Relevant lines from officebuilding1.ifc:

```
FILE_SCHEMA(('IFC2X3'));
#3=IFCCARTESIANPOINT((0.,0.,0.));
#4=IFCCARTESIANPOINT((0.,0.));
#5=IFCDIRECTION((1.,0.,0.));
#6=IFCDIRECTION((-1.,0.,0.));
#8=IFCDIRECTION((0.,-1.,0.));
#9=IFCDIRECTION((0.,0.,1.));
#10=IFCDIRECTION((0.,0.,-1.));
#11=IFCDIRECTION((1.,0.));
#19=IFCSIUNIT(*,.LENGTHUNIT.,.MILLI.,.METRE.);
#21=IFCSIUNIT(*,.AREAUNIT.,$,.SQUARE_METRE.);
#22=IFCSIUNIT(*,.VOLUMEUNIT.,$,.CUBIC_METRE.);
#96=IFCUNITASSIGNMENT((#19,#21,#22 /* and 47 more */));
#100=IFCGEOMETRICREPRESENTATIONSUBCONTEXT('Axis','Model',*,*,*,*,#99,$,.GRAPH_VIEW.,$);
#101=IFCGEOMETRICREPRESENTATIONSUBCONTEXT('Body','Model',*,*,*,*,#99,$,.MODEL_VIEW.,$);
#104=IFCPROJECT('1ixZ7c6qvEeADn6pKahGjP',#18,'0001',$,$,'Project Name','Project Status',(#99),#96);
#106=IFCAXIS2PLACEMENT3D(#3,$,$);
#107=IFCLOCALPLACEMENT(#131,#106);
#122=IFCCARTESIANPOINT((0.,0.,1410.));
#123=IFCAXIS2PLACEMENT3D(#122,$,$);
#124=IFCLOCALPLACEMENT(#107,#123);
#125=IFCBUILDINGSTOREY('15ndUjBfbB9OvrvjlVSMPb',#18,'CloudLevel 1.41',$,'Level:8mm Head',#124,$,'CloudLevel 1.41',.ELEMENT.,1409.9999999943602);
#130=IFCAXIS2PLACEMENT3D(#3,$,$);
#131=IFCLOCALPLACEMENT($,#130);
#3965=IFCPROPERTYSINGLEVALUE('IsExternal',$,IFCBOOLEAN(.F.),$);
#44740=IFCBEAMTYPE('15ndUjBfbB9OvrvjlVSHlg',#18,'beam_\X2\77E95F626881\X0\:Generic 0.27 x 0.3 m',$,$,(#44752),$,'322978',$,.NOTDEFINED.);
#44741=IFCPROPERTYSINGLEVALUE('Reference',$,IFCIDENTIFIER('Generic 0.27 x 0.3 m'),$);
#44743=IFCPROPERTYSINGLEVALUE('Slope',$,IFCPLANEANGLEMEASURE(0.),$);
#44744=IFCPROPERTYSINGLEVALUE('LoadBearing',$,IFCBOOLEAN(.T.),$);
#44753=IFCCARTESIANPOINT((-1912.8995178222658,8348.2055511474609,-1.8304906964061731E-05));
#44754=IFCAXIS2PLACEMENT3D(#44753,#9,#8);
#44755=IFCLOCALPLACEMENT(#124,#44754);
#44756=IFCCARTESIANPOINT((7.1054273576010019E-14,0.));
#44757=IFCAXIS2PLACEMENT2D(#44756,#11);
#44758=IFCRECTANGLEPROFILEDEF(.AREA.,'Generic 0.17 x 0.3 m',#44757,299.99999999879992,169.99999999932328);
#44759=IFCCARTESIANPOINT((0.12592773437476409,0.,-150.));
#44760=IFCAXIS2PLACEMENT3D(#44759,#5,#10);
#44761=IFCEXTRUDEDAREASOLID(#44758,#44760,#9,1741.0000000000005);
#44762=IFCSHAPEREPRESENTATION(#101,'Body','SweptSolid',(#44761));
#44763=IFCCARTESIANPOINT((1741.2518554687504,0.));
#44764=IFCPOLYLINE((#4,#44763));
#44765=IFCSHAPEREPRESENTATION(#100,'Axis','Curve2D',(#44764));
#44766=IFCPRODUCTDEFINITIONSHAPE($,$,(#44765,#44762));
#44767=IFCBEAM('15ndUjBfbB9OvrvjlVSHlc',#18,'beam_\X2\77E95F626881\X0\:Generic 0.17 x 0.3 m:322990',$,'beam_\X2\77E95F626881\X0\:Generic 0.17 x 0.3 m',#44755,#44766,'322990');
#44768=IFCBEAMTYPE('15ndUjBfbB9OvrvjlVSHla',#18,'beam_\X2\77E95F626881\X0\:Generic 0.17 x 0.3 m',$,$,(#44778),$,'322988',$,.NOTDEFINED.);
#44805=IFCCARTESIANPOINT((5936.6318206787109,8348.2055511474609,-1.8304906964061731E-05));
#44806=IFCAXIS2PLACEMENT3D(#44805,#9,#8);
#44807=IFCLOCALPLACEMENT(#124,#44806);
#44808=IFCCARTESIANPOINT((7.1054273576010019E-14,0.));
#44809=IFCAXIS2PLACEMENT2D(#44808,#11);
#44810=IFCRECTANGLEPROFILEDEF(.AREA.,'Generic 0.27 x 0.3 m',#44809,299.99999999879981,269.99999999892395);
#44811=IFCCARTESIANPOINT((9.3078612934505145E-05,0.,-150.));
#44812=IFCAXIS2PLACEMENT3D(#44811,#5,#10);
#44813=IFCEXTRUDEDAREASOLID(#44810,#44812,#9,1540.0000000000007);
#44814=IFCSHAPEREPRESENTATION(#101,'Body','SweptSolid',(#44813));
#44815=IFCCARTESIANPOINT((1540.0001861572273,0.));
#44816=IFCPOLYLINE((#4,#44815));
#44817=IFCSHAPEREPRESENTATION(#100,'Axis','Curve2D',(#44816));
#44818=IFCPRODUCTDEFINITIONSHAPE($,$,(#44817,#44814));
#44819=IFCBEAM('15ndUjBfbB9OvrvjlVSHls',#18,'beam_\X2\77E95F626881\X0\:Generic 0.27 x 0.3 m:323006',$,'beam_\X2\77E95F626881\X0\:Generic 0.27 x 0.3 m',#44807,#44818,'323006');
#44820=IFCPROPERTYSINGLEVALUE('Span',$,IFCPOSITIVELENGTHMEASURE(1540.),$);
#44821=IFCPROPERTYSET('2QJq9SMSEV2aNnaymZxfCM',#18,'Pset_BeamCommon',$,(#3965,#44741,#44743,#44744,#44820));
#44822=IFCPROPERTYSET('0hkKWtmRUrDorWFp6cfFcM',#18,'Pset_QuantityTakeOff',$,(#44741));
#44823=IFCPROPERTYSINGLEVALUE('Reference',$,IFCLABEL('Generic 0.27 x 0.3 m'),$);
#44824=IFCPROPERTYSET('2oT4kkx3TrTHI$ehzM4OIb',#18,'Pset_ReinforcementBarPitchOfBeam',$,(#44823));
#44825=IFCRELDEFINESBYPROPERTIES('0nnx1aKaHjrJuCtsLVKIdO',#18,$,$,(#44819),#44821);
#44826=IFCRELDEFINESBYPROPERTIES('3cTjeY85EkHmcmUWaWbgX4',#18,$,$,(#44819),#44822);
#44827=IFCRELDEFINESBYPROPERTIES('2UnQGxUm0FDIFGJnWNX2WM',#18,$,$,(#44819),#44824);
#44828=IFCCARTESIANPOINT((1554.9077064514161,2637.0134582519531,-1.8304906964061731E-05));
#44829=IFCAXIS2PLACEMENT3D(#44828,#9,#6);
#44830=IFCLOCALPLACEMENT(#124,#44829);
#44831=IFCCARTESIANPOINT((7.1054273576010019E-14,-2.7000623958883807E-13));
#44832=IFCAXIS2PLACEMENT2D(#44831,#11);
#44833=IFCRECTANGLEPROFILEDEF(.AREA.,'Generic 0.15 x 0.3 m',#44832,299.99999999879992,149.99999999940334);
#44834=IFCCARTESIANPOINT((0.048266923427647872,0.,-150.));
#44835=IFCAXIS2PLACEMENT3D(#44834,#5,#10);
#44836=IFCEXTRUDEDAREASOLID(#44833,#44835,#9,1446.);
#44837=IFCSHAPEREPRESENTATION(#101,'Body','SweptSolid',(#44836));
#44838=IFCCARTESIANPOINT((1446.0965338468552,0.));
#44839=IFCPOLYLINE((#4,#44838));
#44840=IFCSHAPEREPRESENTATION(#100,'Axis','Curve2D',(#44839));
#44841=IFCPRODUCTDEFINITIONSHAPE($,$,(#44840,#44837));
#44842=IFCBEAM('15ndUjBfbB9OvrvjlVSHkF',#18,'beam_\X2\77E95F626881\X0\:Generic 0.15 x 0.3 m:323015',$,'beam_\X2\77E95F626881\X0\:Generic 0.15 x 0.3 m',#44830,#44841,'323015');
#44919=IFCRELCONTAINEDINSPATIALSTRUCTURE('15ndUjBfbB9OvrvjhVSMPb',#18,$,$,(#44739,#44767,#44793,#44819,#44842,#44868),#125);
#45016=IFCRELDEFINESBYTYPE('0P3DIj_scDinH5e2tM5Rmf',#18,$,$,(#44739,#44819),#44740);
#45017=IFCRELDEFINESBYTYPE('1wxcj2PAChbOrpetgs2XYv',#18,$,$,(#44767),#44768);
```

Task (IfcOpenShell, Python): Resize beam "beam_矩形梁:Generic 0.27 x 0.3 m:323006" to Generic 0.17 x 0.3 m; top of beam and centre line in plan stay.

```python
import ifcopenshell
import ifcopenshell.api.pset
import ifcopenshell.api.type
import ifcopenshell.util.element
import ifcopenshell.util.representation

model = ifcopenshell.open("officebuilding1.ifc")

member = model.by_id(44819)
source = next(p for p in model.by_type("IfcRectangleProfileDef") if p.ProfileName == "Generic 0.17 x 0.3 m")

body = ifcopenshell.util.representation.get_representation(member, "Model", "Body")
solid = body.Items[0]
old_profile = solid.SweptArea

# Copy the section's sizes but keep this member's own profile position.
profile = ifcopenshell.util.element.copy(model, source)
# Profiles are centred, so shift by half the change in depth to hold the top.
shift = (old_profile.XDim - profile.XDim) / 2
x, y = old_profile.Position.Location.Coordinates
up = (-1.0, 0.0)  # upwards, in the solid's own plane
location = model.createIfcCartesianPoint((x + up[0] * shift, y + up[1] * shift))
profile.Position = model.createIfcAxis2Placement2D(location, old_profile.Position.RefDirection)
solid.SweptArea = profile
if not model.get_total_inverses(old_profile):
    ifcopenshell.util.element.remove_deep2(model, old_profile)

new_type = model.by_guid("15ndUjBfbB9OvrvjlVSHla")
ifcopenshell.api.type.assign_type(
    model, related_objects=[member], relating_type=new_type, should_map_representations=False
)
member.Name = member.Name.replace("Generic 0.27 x 0.3 m", "Generic 0.17 x 0.3 m")
member.ObjectType = "beam_矩形梁:Generic 0.17 x 0.3 m"
pset = model.by_id(ifcopenshell.util.element.get_pset(member, "Pset_BeamCommon", should_inherit=False)["id"])
ifcopenshell.api.pset.edit_pset(model, pset=pset, properties={"Reference": "Generic 0.17 x 0.3 m"})
pset = model.by_id(ifcopenshell.util.element.get_pset(member, "Pset_QuantityTakeOff", should_inherit=False)["id"])
ifcopenshell.api.pset.edit_pset(model, pset=pset, properties={"Reference": "Generic 0.17 x 0.3 m"})
pset = model.by_id(ifcopenshell.util.element.get_pset(member, "Pset_ReinforcementBarPitchOfBeam", should_inherit=False)["id"])
ifcopenshell.api.pset.edit_pset(model, pset=pset, properties={"Reference": "Generic 0.17 x 0.3 m"})

print(solid.SweptArea)

model.write("officebuilding1-out.ifc")
```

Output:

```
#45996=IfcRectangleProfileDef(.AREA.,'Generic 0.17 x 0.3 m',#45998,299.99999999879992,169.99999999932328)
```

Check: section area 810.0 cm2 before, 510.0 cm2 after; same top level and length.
